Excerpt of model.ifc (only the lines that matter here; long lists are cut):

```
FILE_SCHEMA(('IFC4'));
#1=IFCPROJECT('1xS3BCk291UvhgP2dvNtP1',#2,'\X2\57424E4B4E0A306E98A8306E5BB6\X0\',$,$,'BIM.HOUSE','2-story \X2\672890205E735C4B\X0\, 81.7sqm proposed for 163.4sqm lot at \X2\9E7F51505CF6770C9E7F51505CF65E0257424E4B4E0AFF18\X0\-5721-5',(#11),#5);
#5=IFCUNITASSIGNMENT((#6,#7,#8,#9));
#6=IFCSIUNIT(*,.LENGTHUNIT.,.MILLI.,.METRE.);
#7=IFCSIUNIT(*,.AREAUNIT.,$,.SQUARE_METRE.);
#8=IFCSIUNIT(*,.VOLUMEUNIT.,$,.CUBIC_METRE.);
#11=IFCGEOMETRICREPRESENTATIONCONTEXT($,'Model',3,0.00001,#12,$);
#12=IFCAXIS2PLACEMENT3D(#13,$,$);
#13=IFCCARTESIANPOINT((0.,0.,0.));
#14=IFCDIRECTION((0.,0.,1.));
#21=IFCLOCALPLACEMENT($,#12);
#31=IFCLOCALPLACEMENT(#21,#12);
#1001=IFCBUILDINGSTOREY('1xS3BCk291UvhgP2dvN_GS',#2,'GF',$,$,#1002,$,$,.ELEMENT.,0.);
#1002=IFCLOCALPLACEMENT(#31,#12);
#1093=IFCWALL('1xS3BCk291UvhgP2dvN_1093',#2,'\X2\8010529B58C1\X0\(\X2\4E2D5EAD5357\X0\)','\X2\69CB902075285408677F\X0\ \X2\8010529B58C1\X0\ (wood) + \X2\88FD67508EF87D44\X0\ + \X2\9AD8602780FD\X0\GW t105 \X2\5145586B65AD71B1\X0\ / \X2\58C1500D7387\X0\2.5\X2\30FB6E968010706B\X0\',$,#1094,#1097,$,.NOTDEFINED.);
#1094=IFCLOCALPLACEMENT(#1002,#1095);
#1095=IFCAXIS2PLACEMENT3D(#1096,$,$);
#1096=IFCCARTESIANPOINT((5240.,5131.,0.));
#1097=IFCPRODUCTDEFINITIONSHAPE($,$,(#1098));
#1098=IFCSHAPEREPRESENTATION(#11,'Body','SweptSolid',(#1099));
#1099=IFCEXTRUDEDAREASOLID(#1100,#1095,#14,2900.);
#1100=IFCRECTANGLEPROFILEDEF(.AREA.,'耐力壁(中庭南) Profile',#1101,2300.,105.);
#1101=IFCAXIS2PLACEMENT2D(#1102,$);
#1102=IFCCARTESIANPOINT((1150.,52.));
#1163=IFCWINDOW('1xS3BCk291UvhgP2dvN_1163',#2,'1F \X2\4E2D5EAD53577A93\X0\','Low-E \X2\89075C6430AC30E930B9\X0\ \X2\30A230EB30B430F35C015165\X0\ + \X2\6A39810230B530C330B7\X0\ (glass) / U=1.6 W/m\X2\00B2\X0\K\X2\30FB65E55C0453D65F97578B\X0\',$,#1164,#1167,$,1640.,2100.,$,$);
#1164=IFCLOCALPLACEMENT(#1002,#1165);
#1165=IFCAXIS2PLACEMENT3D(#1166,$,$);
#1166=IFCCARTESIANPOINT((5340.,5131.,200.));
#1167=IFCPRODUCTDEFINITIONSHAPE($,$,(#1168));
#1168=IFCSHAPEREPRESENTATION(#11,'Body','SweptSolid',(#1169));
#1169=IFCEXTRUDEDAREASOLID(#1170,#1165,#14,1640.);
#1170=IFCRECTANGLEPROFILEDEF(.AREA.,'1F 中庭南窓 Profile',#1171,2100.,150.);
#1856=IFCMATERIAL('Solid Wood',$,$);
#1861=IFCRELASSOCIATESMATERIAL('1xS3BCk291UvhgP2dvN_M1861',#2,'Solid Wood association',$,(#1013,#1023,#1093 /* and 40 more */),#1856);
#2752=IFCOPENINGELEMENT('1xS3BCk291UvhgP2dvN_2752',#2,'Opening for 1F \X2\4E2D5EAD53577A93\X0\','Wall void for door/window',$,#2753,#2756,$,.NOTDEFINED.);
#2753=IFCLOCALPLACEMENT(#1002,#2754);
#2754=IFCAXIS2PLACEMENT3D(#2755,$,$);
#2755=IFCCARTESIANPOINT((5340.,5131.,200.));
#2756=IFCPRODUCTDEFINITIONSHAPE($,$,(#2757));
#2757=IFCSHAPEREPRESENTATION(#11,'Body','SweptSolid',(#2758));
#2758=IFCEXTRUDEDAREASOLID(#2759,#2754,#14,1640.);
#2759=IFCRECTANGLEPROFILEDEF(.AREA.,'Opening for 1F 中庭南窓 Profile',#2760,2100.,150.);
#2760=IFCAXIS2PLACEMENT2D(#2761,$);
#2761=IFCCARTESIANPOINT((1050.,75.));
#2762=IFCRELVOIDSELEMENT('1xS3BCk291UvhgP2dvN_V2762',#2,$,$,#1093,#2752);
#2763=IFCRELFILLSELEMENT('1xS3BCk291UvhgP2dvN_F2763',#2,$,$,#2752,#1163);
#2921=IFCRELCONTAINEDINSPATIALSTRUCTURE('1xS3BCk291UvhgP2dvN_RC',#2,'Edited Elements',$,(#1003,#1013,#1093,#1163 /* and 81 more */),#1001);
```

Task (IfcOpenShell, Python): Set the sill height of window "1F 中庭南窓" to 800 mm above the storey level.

```python
import numpy as np
import ifcopenshell
import ifcopenshell.api.geometry
import ifcopenshell.geom
import ifcopenshell.util.element
import ifcopenshell.util.placement
import ifcopenshell.util.shape
import ifcopenshell.util.unit

model = ifcopenshell.open("model.ifc")
unit_scale = ifcopenshell.util.unit.calculate_unit_scale(model)

window = model.by_guid("1xS3BCk291UvhgP2dvN_1163")
opening = window.FillsVoids[0].RelatingOpeningElement
storey = ifcopenshell.util.element.get_container(window, ifc_class="IfcBuildingStorey")
level = ifcopenshell.util.placement.get_local_placement(storey.ObjectPlacement)[2, 3]

# The opening's origin need not be at the sill, so measure its lowest point.
shape = ifcopenshell.geom.create_shape(ifcopenshell.geom.settings(), opening)
bottom = ifcopenshell.util.shape.get_shape_bottom_elevation(shape, shape.geometry) / unit_scale
dz = level + 800.0 - bottom

shift = np.array([0.0, 0.0, dz])
# The window is not placed relative to its opening, so move both.
for product in (opening, window):
    matrix = ifcopenshell.util.placement.get_local_placement(product.ObjectPlacement)
    matrix[:3, 3] += shift
    ifcopenshell.api.geometry.edit_object_placement(model, product=product, matrix=matrix, is_si=False)

print(f"moved by {dz * unit_scale:+.3f} m")

model.write("model_updated.ifc")
```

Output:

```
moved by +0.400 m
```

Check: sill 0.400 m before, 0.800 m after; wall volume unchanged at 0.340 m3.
